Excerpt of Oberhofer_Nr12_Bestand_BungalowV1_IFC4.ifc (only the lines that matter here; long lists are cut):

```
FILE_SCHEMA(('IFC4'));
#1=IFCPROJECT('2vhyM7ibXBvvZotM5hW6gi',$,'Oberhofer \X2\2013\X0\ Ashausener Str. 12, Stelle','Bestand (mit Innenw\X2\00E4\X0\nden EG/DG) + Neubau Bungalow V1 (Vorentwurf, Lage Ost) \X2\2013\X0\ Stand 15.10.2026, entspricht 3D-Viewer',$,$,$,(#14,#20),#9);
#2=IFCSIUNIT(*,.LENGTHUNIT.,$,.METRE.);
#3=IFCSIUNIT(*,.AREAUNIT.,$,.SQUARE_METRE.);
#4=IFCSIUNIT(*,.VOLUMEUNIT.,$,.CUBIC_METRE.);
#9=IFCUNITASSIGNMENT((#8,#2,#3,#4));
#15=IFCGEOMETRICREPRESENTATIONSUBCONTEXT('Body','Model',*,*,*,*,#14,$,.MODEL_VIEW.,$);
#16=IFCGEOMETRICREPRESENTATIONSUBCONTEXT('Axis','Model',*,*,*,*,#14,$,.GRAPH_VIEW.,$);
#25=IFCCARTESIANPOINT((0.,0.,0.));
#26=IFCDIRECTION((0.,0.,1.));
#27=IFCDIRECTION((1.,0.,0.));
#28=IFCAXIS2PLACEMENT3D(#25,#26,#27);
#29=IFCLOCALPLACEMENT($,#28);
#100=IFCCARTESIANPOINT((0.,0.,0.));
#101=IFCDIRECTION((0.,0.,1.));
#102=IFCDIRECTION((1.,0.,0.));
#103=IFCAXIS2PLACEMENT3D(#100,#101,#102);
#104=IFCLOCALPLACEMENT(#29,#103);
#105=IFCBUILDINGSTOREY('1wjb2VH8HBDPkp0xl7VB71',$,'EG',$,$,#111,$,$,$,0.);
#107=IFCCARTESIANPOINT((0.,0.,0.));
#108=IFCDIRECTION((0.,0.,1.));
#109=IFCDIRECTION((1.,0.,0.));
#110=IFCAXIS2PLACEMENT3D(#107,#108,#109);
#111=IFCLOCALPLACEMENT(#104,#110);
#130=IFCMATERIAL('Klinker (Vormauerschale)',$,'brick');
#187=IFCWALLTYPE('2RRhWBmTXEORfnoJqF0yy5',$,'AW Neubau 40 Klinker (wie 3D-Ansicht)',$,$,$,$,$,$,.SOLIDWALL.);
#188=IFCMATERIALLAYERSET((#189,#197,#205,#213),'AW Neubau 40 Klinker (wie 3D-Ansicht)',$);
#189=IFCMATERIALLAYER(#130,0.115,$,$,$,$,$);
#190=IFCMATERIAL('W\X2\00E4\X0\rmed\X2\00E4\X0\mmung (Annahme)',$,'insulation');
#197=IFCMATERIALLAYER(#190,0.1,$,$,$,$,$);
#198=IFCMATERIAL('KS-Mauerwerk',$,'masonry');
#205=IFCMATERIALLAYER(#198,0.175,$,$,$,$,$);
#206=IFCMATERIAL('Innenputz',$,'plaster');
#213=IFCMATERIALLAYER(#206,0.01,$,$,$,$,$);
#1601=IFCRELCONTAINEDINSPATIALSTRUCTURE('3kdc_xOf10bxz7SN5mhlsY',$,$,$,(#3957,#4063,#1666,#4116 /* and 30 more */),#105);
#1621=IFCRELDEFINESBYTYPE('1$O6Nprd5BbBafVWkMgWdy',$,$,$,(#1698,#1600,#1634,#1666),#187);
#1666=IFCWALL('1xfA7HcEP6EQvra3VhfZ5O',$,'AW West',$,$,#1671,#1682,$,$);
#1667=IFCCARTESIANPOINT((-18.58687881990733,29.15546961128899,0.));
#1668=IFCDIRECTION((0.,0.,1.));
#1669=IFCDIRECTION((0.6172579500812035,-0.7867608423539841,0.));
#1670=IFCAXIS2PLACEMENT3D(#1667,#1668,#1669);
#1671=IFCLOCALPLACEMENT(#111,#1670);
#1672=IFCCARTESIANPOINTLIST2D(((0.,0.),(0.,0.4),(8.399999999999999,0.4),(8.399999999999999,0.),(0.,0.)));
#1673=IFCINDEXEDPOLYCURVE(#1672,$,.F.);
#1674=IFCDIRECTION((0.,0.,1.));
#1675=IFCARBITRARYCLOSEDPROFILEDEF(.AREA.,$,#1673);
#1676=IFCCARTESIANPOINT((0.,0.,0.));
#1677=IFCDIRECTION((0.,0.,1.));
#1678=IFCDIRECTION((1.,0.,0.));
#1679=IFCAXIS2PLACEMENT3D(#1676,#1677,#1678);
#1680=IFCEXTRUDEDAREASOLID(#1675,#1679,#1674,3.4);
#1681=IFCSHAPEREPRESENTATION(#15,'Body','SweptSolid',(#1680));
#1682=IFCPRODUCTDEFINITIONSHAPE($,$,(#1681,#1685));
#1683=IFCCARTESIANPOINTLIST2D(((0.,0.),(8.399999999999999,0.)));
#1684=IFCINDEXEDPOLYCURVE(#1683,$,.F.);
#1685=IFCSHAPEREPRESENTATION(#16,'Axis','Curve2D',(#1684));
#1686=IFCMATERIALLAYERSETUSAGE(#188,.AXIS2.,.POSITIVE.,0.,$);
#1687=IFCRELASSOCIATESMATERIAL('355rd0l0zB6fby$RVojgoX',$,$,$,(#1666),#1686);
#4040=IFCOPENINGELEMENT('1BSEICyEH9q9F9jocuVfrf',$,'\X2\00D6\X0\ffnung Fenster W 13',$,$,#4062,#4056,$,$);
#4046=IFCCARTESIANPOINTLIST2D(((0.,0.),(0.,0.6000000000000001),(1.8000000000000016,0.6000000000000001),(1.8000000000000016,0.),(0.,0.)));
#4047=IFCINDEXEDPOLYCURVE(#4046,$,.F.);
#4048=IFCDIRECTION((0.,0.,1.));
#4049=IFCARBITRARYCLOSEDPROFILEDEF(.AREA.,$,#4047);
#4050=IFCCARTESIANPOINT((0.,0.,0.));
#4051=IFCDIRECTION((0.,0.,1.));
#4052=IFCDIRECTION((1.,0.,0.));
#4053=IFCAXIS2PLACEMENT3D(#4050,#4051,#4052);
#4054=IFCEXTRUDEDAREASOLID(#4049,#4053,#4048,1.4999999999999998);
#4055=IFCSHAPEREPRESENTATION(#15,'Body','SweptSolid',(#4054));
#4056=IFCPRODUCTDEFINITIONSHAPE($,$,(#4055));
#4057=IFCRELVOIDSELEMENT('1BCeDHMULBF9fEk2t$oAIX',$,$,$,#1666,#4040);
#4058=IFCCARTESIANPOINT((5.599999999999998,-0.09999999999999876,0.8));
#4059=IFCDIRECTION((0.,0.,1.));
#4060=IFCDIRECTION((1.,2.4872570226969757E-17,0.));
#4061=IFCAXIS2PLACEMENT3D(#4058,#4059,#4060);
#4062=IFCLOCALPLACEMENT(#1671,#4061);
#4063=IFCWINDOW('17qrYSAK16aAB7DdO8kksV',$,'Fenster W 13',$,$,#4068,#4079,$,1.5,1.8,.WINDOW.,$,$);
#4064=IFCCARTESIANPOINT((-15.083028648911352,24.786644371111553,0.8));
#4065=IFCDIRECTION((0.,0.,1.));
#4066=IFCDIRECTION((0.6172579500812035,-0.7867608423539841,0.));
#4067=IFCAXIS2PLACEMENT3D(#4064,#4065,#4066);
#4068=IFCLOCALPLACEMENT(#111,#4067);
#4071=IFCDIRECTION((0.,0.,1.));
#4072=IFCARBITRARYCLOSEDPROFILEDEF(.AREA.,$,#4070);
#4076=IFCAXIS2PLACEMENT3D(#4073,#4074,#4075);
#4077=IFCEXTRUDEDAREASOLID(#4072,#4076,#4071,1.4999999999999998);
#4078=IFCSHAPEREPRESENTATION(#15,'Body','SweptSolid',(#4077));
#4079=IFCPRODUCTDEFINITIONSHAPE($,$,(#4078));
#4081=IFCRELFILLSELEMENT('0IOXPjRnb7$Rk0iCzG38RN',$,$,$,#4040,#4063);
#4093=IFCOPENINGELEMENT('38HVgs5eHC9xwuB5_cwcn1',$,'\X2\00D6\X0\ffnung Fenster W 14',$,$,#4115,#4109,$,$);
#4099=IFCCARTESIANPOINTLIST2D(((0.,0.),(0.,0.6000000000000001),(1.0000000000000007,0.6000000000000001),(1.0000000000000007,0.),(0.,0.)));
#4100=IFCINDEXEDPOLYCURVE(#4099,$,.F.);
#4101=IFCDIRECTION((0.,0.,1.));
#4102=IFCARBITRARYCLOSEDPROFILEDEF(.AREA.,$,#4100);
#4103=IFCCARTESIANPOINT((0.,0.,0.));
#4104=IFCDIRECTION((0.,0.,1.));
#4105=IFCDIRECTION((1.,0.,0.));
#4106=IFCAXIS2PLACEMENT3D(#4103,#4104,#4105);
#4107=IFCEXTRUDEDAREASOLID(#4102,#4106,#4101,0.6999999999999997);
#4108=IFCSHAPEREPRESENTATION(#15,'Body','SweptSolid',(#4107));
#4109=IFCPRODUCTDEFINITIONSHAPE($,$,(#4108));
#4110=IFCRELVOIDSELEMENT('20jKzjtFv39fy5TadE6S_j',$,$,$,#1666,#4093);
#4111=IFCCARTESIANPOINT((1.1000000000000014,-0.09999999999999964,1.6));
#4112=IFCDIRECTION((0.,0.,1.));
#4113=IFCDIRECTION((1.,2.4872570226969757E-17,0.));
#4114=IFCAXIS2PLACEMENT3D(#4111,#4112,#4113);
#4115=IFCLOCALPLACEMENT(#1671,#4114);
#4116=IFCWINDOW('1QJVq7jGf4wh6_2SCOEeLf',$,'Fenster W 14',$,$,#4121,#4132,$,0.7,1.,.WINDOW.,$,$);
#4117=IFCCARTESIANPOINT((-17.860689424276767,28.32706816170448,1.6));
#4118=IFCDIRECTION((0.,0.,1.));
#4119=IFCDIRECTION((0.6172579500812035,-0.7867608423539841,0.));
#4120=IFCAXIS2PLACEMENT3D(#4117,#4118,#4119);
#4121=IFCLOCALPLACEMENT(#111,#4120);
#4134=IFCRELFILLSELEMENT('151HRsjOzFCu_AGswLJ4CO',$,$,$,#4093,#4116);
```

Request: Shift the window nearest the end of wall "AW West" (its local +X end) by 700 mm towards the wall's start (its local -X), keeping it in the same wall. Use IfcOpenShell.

```python
import ifcopenshell
import ifcopenshell.api.geometry
import ifcopenshell.util.placement

model = ifcopenshell.open("Oberhofer_Nr12_Bestand_BungalowV1_IFC4.ifc")

window = model.by_guid("17qrYSAK16aAB7DdO8kksV")
opening = window.FillsVoids[0].RelatingOpeningElement
wall = opening.VoidsElements[0].RelatingBuildingElement

wall_matrix = ifcopenshell.util.placement.get_local_placement(wall.ObjectPlacement)
shift = wall_matrix[:3, 0] * -0.7
before = ifcopenshell.util.placement.get_local_placement(window.ObjectPlacement)[:3, 3].copy()

# The window is not placed relative to its opening, so move both.
for product in (opening, window):
    matrix = ifcopenshell.util.placement.get_local_placement(product.ObjectPlacement)
    matrix[:3, 3] += shift
    ifcopenshell.api.geometry.edit_object_placement(model, product=product, matrix=matrix, is_si=False)

after = ifcopenshell.util.placement.get_local_placement(window.ObjectPlacement)[:3, 3]
print("window moved by", (after - before).round(3) + 0.0)

model.write("Oberhofer_Nr12_Bestand_BungalowV1_IFC4_updated.ifc")
```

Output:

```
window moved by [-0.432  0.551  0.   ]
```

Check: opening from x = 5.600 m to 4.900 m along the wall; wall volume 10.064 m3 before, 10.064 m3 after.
